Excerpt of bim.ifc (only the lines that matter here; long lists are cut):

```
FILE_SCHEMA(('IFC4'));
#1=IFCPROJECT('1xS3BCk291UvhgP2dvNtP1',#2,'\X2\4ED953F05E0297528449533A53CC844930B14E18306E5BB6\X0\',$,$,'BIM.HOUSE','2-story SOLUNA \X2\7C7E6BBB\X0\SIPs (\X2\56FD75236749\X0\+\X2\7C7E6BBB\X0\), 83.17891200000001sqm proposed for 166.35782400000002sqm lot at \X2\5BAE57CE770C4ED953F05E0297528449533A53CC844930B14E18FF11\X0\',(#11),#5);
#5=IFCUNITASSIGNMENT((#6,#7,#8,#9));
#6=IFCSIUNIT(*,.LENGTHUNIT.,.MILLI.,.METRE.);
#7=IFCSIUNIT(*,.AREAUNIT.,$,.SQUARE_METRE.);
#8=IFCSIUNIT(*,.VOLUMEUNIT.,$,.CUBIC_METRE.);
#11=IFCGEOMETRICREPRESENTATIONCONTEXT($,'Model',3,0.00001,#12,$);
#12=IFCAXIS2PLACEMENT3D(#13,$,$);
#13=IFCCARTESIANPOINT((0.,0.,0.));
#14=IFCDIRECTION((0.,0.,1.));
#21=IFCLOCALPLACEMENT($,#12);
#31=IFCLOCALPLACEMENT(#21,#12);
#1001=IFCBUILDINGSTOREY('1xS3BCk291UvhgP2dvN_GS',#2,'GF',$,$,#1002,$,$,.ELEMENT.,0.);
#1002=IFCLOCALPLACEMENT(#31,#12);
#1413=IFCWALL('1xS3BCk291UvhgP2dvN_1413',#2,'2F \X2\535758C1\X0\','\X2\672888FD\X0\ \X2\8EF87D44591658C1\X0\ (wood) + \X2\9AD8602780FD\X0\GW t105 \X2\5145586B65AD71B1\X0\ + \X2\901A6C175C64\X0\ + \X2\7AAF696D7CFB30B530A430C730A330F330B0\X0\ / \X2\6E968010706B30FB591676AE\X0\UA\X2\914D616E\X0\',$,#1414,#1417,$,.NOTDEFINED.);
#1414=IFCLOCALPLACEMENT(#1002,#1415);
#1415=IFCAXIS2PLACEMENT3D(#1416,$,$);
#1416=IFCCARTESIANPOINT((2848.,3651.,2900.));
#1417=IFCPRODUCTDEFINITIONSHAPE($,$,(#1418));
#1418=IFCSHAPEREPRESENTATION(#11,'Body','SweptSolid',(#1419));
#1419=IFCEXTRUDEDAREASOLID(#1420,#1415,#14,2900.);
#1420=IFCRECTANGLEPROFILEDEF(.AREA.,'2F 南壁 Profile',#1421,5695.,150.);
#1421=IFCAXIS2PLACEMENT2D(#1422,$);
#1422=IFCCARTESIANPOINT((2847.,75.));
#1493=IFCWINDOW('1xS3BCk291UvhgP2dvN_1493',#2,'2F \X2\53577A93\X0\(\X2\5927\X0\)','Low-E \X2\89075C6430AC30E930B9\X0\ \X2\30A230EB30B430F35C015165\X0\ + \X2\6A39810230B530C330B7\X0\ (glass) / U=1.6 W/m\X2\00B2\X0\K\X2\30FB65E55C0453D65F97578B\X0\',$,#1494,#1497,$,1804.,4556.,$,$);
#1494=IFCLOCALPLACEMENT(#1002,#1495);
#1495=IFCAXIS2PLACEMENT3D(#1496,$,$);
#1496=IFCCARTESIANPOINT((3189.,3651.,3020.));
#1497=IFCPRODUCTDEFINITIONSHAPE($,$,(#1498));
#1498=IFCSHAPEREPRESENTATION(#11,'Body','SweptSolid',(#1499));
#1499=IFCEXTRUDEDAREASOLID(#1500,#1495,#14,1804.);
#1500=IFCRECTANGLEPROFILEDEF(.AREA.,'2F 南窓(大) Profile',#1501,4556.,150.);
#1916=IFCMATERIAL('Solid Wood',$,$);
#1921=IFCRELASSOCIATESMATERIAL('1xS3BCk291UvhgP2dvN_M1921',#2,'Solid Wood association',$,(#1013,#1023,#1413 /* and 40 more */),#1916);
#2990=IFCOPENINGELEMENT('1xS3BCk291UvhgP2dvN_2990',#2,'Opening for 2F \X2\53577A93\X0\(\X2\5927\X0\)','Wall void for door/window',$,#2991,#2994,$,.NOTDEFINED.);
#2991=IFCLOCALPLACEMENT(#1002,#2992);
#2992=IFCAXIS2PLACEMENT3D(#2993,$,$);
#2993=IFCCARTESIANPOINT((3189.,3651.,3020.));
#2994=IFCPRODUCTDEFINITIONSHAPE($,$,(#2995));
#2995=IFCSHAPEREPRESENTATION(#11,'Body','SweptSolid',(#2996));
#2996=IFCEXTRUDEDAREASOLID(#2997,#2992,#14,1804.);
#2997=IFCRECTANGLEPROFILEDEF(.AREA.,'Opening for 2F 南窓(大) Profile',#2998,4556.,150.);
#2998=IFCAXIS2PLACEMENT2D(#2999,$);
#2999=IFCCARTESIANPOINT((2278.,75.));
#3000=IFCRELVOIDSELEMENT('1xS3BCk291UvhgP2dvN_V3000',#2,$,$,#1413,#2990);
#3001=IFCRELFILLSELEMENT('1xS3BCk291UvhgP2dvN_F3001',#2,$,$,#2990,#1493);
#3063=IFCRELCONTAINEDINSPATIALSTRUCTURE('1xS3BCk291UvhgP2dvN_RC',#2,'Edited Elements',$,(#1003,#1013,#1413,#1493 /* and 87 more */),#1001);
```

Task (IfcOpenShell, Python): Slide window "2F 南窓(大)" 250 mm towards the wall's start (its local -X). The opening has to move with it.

```python
import ifcopenshell
import ifcopenshell.api.geometry
import ifcopenshell.util.placement
import ifcopenshell.util.unit

model = ifcopenshell.open("bim.ifc")
unit_scale = ifcopenshell.util.unit.calculate_unit_scale(model)

window = model.by_guid("1xS3BCk291UvhgP2dvN_1493")
opening = window.FillsVoids[0].RelatingOpeningElement
wall = opening.VoidsElements[0].RelatingBuildingElement

wall_matrix = ifcopenshell.util.placement.get_local_placement(wall.ObjectPlacement)
shift = wall_matrix[:3, 0] * -0.25 / unit_scale
before = ifcopenshell.util.placement.get_local_placement(window.ObjectPlacement)[:3, 3].copy()

# The window is not placed relative to its opening, so move both.
for product in (opening, window):
    matrix = ifcopenshell.util.placement.get_local_placement(product.ObjectPlacement)
    matrix[:3, 3] += shift
    ifcopenshell.api.geometry.edit_object_placement(model, product=product, matrix=matrix, is_si=False)

after = ifcopenshell.util.placement.get_local_placement(window.ObjectPlacement)[:3, 3]
print("window moved by", (after - before).round(3) + 0.0)

model.write("bim_rev.ifc")
```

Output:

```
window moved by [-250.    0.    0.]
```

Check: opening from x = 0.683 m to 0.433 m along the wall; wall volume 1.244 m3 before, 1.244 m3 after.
